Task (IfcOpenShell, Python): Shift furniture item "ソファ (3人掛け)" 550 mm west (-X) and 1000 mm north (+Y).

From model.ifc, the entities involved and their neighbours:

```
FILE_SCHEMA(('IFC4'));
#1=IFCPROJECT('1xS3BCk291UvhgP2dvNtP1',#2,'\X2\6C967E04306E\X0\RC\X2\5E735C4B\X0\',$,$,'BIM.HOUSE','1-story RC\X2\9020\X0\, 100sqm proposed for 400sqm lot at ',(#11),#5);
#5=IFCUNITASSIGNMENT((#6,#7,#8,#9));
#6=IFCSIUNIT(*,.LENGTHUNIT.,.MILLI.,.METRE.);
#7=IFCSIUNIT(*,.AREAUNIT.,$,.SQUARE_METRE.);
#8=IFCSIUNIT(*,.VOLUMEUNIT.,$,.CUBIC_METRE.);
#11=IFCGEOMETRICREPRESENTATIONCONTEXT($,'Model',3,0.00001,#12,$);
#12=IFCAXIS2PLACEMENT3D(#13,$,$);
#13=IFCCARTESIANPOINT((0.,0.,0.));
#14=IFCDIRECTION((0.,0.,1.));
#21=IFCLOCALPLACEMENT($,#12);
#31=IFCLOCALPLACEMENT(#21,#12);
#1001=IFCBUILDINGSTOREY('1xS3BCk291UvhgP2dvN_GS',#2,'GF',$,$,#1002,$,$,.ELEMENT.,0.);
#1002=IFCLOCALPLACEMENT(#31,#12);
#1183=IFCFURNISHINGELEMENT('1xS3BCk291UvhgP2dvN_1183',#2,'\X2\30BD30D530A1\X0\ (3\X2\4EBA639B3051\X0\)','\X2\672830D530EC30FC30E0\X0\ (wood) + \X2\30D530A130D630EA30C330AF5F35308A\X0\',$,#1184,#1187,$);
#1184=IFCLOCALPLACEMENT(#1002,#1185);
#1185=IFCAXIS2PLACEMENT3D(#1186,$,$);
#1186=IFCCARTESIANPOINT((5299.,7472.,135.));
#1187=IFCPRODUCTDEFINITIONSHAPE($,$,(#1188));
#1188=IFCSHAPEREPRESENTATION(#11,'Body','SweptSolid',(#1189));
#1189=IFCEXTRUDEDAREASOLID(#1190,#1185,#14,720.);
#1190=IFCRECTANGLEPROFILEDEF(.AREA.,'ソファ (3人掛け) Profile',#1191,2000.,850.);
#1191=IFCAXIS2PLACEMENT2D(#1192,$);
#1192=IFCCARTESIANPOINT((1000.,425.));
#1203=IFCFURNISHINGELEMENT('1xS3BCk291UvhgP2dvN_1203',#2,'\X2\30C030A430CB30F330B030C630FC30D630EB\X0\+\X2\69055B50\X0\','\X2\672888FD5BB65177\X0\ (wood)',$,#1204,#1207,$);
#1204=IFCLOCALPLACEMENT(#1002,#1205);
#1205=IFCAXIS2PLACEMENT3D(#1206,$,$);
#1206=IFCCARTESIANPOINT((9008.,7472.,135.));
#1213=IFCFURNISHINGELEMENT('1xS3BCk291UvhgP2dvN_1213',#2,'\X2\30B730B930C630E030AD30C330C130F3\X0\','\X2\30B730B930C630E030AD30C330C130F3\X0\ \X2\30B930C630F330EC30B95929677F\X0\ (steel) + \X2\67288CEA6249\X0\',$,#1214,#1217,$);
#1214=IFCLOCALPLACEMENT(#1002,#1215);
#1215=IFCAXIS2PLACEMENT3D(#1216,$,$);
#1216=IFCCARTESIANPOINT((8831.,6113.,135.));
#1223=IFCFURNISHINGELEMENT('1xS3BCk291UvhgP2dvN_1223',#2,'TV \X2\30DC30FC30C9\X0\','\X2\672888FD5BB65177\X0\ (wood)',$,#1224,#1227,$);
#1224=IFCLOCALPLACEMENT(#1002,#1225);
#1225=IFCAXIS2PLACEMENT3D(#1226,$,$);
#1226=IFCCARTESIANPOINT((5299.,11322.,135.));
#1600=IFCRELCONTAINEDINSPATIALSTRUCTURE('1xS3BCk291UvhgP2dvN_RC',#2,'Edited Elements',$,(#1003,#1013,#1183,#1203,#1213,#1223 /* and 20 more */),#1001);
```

```python
import ifcopenshell
import ifcopenshell.api.geometry
import ifcopenshell.util.placement
import ifcopenshell.util.unit

model = ifcopenshell.open("model.ifc")
unit_scale = ifcopenshell.util.unit.calculate_unit_scale(model)

item = model.by_guid("1xS3BCk291UvhgP2dvN_1183")
matrix = ifcopenshell.util.placement.get_local_placement(item.ObjectPlacement)
matrix[0, 3] -= 0.55 / unit_scale
matrix[1, 3] += 1 / unit_scale
ifcopenshell.api.geometry.edit_object_placement(model, product=item, matrix=matrix, is_si=False)

print(ifcopenshell.util.placement.get_local_placement(item.ObjectPlacement).round(3) + 0.0)

model.write("model_v2.ifc")
```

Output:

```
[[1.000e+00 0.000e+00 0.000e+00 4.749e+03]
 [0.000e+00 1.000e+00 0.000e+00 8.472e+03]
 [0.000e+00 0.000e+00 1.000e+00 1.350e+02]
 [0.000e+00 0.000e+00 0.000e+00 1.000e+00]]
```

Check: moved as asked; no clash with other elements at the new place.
